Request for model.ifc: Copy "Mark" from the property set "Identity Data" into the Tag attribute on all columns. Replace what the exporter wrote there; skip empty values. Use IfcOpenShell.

First a look at what the model holds.

```python
import ifcopenshell
import ifcopenshell.util.element

model = ifcopenshell.open("model.ifc")
print(model.schema)
columns = model.by_type("IfcColumn")
print(len(columns), "columns")
for e in columns[:8]:
    source = ifcopenshell.util.element.get_pset(e, "Identity Data", "Mark")
    target = e.Tag
    print(e.id(), repr(source), repr(target), sep=" | ")
```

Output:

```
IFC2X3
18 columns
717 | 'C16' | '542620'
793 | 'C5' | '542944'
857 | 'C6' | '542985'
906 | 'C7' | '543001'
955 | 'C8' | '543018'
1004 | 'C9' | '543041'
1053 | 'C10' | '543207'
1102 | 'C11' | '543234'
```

```python
import ifcopenshell
import ifcopenshell.util.element

model = ifcopenshell.open("model.ifc")

count = 0
for e in model.by_type("IfcColumn"):
    value = ifcopenshell.util.element.get_pset(e, "Identity Data", "Mark")
    current = e.Tag
    if not value or not value.strip() or current == value:
        continue
    e.Tag = value
    count += 1

print(count, "columns updated")

model.write("model_updated.ifc")
```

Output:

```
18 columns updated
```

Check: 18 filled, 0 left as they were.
